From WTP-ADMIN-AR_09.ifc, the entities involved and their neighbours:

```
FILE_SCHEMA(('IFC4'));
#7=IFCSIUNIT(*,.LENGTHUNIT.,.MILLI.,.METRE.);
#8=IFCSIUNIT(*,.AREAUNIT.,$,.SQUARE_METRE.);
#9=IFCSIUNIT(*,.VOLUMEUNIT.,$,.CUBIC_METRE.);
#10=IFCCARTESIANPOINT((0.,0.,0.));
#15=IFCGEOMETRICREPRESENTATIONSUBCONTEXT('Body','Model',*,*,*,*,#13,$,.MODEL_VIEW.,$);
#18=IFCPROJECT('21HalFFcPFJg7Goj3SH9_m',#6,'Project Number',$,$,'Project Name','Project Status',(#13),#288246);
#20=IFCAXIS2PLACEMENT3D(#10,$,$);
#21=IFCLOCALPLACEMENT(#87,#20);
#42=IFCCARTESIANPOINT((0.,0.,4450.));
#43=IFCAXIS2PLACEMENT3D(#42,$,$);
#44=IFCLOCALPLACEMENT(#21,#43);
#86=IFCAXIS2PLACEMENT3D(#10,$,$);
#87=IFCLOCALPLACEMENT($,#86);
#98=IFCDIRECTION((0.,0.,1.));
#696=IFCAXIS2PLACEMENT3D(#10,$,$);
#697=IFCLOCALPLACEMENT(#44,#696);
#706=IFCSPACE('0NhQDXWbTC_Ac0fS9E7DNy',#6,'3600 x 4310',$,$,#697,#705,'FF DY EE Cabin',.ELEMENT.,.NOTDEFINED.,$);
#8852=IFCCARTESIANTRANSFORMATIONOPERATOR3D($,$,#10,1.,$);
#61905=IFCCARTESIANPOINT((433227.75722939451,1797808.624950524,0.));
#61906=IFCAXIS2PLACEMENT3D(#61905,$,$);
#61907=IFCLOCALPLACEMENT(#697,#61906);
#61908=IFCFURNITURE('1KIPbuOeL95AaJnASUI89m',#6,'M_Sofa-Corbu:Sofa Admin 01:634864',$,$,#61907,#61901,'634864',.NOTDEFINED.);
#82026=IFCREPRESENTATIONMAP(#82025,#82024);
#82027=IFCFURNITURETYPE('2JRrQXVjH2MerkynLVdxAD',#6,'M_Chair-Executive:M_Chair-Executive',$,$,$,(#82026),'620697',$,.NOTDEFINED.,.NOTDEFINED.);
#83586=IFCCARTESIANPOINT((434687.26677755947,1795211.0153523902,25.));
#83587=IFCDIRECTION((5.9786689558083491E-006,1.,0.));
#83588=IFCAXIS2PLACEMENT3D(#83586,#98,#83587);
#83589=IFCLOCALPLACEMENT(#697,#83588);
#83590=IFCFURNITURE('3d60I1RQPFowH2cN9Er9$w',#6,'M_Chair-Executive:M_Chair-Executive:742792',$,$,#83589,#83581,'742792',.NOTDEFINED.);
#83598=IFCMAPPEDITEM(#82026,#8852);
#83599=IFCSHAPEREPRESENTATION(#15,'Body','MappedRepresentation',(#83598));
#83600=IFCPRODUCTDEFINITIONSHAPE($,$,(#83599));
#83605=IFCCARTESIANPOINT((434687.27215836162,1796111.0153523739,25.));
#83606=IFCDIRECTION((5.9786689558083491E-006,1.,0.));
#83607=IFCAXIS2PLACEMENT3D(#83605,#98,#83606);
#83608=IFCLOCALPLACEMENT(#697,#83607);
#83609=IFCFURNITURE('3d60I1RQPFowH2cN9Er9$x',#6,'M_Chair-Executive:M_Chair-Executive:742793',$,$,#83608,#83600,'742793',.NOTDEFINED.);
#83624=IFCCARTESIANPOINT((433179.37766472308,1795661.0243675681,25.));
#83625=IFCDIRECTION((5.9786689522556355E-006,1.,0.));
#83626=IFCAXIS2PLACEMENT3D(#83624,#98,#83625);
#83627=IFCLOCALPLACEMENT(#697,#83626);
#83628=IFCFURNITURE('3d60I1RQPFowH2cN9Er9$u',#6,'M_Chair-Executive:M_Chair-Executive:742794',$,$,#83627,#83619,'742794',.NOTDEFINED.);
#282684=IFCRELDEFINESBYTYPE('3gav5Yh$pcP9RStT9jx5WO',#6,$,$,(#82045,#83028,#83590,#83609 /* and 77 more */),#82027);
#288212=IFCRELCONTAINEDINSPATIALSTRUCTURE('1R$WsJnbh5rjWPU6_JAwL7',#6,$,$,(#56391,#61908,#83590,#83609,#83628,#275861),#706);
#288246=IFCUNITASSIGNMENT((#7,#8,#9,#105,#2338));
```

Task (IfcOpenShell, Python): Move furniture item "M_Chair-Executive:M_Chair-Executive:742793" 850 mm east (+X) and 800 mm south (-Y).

```python
import ifcopenshell
import ifcopenshell.api.geometry
import ifcopenshell.util.placement

model = ifcopenshell.open("WTP-ADMIN-AR_09.ifc")

item = model.by_guid("3d60I1RQPFowH2cN9Er9$x")
matrix = ifcopenshell.util.placement.get_local_placement(item.ObjectPlacement)
matrix[0, 3] += 850.0
matrix[1, 3] -= 800.0
ifcopenshell.api.geometry.edit_object_placement(model, product=item, matrix=matrix, is_si=False)

print(ifcopenshell.util.placement.get_local_placement(item.ObjectPlacement).round(3) + 0.0)

model.write("WTP-ADMIN-AR_09_rev.ifc")
```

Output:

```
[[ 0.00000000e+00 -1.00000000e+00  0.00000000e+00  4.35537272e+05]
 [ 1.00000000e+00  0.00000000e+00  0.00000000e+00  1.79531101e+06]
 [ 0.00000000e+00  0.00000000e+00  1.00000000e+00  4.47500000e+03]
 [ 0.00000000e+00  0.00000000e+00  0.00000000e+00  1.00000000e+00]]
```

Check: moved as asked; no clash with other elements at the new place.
